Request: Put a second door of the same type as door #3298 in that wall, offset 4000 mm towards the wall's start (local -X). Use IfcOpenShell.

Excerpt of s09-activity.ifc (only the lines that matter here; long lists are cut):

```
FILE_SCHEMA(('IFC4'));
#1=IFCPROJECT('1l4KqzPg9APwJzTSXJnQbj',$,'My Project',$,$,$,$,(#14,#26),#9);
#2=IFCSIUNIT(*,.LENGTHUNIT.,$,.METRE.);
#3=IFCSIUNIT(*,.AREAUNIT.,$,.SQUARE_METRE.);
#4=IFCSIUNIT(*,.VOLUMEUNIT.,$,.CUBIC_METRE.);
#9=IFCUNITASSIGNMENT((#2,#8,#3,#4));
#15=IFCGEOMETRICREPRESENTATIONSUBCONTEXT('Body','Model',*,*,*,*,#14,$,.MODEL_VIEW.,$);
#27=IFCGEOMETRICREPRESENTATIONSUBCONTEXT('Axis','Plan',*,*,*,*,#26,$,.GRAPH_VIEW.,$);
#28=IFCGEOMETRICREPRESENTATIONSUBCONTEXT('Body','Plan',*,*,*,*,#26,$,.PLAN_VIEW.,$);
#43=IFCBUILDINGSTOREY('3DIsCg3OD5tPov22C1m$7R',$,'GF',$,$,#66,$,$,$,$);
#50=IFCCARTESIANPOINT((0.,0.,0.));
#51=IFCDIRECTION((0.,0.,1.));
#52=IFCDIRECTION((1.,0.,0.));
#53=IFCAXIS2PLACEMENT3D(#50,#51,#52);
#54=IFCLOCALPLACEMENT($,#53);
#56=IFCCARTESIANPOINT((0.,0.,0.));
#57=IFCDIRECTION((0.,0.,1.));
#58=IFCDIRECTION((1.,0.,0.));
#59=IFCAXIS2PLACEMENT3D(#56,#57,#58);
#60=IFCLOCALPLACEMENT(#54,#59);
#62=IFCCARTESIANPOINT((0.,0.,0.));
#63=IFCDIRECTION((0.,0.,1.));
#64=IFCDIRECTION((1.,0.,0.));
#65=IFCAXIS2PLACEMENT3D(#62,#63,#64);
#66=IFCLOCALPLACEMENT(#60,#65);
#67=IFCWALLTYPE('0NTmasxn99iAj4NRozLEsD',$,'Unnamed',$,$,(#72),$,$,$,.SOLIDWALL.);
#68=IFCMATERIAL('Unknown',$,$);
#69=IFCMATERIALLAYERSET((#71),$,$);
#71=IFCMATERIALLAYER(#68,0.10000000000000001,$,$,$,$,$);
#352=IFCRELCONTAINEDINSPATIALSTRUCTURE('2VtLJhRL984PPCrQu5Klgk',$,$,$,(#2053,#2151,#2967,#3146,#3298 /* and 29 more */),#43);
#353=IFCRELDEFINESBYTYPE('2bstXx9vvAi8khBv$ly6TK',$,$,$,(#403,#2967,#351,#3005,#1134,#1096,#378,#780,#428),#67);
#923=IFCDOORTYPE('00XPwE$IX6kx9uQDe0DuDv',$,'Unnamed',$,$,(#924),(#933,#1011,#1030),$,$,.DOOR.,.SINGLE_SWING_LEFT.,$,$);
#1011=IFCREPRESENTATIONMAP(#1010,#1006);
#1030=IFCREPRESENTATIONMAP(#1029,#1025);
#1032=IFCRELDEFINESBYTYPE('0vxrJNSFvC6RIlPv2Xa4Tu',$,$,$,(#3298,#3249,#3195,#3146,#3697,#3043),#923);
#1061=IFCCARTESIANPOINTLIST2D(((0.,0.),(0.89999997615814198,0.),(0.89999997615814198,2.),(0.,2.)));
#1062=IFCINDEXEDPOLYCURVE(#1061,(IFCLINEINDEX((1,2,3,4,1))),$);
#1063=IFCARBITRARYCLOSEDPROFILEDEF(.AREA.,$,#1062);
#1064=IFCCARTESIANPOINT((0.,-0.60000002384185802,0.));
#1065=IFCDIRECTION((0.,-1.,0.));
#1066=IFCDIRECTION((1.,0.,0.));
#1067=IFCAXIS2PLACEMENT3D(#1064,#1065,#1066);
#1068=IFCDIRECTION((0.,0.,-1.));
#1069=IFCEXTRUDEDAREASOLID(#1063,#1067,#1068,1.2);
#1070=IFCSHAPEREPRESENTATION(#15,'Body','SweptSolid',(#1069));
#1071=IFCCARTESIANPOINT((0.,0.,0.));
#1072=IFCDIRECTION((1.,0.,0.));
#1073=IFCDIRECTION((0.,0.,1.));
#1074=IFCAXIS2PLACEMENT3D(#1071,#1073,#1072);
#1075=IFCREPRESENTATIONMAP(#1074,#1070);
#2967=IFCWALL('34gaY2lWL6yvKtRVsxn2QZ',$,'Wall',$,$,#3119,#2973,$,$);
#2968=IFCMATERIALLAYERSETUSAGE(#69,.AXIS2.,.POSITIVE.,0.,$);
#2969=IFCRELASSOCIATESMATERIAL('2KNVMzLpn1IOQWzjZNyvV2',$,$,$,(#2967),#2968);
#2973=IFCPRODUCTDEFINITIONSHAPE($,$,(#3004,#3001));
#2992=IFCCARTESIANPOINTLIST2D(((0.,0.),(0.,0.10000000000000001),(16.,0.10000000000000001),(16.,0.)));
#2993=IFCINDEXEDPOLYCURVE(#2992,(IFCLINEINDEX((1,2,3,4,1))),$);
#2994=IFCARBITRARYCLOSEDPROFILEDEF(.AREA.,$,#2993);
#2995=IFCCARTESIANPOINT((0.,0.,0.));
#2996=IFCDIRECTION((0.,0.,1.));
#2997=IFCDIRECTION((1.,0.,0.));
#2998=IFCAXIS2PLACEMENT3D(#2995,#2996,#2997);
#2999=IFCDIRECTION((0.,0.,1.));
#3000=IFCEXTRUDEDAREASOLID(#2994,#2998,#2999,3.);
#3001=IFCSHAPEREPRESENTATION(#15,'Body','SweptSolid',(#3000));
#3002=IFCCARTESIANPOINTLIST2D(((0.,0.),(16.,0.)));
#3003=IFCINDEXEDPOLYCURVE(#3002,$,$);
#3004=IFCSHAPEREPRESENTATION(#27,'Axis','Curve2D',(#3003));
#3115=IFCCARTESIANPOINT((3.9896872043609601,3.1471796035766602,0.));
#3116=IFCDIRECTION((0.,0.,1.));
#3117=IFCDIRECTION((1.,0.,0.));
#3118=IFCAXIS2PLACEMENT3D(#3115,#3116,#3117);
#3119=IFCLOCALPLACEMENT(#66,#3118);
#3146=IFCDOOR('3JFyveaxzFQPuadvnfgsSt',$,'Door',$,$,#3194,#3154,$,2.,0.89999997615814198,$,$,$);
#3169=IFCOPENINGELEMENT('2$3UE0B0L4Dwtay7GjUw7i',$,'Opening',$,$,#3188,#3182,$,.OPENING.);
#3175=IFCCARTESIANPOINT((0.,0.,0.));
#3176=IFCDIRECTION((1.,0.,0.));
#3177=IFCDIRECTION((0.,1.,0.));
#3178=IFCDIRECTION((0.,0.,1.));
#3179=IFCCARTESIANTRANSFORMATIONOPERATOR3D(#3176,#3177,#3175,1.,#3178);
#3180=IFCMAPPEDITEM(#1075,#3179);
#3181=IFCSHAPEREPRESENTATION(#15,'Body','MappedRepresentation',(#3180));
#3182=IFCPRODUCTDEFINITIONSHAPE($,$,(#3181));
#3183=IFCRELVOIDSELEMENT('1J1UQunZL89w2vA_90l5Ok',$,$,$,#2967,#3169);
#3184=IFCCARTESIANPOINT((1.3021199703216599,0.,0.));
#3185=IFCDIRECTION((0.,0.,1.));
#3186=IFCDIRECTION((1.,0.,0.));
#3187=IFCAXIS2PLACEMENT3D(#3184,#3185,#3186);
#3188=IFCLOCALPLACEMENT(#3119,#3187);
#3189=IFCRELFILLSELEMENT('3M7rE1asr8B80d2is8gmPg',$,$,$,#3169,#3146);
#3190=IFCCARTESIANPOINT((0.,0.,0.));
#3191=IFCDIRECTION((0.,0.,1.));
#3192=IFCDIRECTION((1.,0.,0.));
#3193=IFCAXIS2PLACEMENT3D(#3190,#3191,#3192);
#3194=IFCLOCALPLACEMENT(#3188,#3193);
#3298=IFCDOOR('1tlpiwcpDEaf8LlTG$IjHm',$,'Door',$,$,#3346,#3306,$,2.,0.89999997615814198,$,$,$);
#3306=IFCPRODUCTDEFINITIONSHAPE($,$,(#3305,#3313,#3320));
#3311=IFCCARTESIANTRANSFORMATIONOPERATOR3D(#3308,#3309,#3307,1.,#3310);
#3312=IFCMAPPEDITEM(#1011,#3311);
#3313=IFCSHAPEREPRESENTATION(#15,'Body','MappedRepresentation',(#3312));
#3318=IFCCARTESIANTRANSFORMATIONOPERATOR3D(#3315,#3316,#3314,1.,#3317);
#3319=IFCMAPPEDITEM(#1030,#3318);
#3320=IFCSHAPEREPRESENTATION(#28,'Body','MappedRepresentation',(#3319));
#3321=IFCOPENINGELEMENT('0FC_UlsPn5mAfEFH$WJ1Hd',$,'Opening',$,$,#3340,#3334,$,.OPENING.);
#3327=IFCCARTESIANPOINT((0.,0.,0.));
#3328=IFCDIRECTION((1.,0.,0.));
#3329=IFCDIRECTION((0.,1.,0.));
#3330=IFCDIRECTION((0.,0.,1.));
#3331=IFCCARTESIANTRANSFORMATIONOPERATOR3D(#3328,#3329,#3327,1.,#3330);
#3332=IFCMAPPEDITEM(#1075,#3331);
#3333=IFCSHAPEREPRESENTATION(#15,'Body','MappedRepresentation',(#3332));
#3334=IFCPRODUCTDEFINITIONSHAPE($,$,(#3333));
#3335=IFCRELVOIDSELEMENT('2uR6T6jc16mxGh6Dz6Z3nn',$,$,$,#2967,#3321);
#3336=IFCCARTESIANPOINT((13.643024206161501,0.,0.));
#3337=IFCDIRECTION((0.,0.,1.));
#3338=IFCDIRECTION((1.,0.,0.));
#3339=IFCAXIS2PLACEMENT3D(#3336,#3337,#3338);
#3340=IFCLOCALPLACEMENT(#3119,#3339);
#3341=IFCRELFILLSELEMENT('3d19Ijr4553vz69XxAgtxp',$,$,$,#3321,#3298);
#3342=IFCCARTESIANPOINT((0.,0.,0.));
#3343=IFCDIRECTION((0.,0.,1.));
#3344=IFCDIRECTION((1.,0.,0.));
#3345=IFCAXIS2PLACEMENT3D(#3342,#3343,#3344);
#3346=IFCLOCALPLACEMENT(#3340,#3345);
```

```python
import ifcopenshell
import ifcopenshell.api.feature
import ifcopenshell.api.geometry
import ifcopenshell.api.root
import ifcopenshell.geom
import ifcopenshell.util.element
import ifcopenshell.util.placement
import ifcopenshell.util.shape

model = ifcopenshell.open("s09-activity.ifc")
settings = ifcopenshell.geom.settings()


def volume(element):
    """Net volume in cubic metres, openings subtracted."""
    shape = ifcopenshell.geom.create_shape(settings, element)
    return ifcopenshell.util.shape.get_volume(shape.geometry)


door = model.by_guid("1tlpiwcpDEaf8LlTG$IjHm")
opening = door.FillsVoids[0].RelatingOpeningElement
wall = opening.VoidsElements[0].RelatingBuildingElement
before = volume(wall)
shift = ifcopenshell.util.placement.get_local_placement(wall.ObjectPlacement)[:3, 0] * -4.0

# copy_class copies the void relationship, type, container and properties, but no geometry.
new_opening = ifcopenshell.api.root.copy_class(model, product=opening)
new_opening.Representation = ifcopenshell.util.element.copy_deep(
    model, opening.Representation, exclude=["IfcGeometricRepresentationContext", "IfcRepresentationMap"]
)
new_door = ifcopenshell.api.root.copy_class(model, product=door)
new_door.Representation = ifcopenshell.util.element.copy_deep(
    model, door.Representation, exclude=["IfcGeometricRepresentationContext", "IfcRepresentationMap"]
)
ifcopenshell.api.feature.add_filling(model, opening=new_opening, element=new_door)

for old, new in ((opening, new_opening), (door, new_door)):
    matrix = ifcopenshell.util.placement.get_local_placement(old.ObjectPlacement)
    matrix[:3, 3] += shift
    ifcopenshell.api.geometry.edit_object_placement(model, product=new, matrix=matrix, is_si=False)

after = volume(wall)

print(f"wall volume {before:.3f} -> {after:.3f} m3")

model.write("s09-activity_v2.ifc")
```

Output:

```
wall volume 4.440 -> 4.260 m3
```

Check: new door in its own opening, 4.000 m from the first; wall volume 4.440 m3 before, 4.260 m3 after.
